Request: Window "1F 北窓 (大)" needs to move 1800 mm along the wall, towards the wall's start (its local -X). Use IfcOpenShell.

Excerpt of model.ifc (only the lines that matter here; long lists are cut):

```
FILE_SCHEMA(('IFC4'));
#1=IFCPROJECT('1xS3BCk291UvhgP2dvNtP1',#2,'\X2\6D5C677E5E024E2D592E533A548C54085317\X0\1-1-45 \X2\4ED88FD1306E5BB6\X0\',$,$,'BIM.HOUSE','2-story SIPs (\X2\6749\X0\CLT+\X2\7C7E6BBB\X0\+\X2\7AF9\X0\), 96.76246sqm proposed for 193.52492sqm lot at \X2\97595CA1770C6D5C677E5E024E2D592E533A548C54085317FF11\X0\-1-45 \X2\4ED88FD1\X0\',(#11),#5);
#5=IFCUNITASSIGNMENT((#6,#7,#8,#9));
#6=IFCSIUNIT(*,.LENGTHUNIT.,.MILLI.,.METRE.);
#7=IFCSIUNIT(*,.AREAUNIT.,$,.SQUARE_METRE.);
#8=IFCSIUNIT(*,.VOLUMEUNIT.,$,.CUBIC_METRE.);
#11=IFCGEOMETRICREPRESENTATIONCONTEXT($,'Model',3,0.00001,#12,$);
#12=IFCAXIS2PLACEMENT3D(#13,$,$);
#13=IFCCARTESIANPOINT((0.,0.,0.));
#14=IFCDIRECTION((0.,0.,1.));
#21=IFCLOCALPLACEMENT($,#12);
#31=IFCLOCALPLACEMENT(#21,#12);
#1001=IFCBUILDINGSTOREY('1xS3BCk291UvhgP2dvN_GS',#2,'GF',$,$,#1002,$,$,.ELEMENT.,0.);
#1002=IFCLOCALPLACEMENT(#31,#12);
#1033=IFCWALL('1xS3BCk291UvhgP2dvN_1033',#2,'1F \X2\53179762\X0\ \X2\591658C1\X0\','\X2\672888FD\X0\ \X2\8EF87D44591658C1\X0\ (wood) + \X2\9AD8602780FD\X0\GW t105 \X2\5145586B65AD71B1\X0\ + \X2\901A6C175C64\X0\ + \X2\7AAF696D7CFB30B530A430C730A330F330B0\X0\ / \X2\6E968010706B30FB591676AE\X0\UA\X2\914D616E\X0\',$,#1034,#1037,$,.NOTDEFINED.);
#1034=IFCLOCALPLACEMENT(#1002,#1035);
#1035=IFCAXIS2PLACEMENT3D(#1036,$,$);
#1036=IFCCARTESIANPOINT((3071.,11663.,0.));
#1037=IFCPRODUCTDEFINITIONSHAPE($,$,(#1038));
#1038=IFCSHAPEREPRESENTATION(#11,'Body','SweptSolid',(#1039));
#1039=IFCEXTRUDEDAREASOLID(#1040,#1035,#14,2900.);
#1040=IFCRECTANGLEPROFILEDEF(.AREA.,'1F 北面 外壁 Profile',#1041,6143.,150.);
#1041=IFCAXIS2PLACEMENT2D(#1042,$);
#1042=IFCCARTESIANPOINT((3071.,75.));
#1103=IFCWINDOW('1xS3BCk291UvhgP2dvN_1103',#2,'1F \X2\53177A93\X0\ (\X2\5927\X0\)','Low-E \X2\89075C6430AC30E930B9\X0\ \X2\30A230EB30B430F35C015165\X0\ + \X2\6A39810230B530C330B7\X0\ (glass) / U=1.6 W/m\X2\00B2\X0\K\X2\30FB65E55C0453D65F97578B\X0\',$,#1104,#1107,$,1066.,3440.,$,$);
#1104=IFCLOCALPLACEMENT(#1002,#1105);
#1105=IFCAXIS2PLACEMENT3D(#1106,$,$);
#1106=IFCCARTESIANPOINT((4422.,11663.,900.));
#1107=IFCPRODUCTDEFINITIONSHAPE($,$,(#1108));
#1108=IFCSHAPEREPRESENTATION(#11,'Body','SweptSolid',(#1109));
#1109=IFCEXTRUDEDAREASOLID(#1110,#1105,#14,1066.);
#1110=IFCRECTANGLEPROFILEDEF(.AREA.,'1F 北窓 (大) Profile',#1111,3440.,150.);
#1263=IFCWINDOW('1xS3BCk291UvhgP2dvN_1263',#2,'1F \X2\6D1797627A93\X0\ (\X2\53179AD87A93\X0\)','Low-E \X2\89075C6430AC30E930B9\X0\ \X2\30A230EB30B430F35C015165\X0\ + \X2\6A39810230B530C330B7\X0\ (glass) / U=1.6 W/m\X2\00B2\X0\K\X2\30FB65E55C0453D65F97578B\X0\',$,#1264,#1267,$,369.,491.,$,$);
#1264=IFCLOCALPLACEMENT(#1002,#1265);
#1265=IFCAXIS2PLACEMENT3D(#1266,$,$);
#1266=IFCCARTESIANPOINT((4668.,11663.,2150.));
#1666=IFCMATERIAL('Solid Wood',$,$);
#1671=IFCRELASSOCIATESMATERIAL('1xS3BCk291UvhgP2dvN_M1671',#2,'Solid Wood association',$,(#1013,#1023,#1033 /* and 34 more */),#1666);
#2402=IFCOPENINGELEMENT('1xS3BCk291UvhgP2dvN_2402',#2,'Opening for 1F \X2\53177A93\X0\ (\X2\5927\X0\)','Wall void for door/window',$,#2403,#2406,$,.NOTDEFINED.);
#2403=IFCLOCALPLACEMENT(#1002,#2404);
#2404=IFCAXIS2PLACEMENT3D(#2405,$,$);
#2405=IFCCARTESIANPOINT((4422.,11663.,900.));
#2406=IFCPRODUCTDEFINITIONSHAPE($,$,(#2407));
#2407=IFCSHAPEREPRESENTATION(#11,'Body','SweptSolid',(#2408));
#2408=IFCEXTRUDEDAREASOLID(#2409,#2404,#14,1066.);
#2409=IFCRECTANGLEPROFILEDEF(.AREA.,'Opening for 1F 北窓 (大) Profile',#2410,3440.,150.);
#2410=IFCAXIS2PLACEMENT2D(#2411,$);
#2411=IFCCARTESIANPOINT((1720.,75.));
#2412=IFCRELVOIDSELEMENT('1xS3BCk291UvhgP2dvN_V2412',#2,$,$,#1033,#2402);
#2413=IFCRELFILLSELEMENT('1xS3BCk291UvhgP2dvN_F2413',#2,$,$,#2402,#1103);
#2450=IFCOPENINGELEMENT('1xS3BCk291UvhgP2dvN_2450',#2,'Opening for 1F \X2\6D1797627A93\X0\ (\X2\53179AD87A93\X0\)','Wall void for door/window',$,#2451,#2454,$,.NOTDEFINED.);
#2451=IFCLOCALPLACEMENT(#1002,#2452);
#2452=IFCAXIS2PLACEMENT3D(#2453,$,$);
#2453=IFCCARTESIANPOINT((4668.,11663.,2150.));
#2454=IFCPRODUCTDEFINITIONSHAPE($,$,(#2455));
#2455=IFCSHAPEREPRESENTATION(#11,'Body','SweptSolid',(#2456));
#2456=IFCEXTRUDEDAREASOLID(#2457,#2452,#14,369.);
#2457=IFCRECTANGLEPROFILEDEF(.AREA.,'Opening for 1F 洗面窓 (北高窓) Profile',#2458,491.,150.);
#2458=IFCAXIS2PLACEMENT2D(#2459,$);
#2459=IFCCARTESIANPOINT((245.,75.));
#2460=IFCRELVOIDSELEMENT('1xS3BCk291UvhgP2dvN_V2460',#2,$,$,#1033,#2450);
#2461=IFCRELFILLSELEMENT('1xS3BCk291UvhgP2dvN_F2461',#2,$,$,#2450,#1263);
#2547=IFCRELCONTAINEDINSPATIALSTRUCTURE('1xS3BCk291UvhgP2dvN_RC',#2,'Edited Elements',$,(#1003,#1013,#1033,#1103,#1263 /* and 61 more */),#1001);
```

```python
import ifcopenshell
import ifcopenshell.api.geometry
import ifcopenshell.util.placement

model = ifcopenshell.open("model.ifc")

window = model.by_guid("1xS3BCk291UvhgP2dvN_1103")
opening = window.FillsVoids[0].RelatingOpeningElement
wall = opening.VoidsElements[0].RelatingBuildingElement

wall_matrix = ifcopenshell.util.placement.get_local_placement(wall.ObjectPlacement)
shift = wall_matrix[:3, 0] * -1800.0
before = ifcopenshell.util.placement.get_local_placement(window.ObjectPlacement)[:3, 3].copy()

# The window is not placed relative to its opening, so move both.
for product in (opening, window):
    matrix = ifcopenshell.util.placement.get_local_placement(product.ObjectPlacement)
    matrix[:3, 3] += shift
    ifcopenshell.api.geometry.edit_object_placement(model, product=product, matrix=matrix, is_si=False)

after = ifcopenshell.util.placement.get_local_placement(window.ObjectPlacement)[:3, 3]
print("window moved by", (after - before).round(3) + 0.0)

model.write("model_rev.ifc")
```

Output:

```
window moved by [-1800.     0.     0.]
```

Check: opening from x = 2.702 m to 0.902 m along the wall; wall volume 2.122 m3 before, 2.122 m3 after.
